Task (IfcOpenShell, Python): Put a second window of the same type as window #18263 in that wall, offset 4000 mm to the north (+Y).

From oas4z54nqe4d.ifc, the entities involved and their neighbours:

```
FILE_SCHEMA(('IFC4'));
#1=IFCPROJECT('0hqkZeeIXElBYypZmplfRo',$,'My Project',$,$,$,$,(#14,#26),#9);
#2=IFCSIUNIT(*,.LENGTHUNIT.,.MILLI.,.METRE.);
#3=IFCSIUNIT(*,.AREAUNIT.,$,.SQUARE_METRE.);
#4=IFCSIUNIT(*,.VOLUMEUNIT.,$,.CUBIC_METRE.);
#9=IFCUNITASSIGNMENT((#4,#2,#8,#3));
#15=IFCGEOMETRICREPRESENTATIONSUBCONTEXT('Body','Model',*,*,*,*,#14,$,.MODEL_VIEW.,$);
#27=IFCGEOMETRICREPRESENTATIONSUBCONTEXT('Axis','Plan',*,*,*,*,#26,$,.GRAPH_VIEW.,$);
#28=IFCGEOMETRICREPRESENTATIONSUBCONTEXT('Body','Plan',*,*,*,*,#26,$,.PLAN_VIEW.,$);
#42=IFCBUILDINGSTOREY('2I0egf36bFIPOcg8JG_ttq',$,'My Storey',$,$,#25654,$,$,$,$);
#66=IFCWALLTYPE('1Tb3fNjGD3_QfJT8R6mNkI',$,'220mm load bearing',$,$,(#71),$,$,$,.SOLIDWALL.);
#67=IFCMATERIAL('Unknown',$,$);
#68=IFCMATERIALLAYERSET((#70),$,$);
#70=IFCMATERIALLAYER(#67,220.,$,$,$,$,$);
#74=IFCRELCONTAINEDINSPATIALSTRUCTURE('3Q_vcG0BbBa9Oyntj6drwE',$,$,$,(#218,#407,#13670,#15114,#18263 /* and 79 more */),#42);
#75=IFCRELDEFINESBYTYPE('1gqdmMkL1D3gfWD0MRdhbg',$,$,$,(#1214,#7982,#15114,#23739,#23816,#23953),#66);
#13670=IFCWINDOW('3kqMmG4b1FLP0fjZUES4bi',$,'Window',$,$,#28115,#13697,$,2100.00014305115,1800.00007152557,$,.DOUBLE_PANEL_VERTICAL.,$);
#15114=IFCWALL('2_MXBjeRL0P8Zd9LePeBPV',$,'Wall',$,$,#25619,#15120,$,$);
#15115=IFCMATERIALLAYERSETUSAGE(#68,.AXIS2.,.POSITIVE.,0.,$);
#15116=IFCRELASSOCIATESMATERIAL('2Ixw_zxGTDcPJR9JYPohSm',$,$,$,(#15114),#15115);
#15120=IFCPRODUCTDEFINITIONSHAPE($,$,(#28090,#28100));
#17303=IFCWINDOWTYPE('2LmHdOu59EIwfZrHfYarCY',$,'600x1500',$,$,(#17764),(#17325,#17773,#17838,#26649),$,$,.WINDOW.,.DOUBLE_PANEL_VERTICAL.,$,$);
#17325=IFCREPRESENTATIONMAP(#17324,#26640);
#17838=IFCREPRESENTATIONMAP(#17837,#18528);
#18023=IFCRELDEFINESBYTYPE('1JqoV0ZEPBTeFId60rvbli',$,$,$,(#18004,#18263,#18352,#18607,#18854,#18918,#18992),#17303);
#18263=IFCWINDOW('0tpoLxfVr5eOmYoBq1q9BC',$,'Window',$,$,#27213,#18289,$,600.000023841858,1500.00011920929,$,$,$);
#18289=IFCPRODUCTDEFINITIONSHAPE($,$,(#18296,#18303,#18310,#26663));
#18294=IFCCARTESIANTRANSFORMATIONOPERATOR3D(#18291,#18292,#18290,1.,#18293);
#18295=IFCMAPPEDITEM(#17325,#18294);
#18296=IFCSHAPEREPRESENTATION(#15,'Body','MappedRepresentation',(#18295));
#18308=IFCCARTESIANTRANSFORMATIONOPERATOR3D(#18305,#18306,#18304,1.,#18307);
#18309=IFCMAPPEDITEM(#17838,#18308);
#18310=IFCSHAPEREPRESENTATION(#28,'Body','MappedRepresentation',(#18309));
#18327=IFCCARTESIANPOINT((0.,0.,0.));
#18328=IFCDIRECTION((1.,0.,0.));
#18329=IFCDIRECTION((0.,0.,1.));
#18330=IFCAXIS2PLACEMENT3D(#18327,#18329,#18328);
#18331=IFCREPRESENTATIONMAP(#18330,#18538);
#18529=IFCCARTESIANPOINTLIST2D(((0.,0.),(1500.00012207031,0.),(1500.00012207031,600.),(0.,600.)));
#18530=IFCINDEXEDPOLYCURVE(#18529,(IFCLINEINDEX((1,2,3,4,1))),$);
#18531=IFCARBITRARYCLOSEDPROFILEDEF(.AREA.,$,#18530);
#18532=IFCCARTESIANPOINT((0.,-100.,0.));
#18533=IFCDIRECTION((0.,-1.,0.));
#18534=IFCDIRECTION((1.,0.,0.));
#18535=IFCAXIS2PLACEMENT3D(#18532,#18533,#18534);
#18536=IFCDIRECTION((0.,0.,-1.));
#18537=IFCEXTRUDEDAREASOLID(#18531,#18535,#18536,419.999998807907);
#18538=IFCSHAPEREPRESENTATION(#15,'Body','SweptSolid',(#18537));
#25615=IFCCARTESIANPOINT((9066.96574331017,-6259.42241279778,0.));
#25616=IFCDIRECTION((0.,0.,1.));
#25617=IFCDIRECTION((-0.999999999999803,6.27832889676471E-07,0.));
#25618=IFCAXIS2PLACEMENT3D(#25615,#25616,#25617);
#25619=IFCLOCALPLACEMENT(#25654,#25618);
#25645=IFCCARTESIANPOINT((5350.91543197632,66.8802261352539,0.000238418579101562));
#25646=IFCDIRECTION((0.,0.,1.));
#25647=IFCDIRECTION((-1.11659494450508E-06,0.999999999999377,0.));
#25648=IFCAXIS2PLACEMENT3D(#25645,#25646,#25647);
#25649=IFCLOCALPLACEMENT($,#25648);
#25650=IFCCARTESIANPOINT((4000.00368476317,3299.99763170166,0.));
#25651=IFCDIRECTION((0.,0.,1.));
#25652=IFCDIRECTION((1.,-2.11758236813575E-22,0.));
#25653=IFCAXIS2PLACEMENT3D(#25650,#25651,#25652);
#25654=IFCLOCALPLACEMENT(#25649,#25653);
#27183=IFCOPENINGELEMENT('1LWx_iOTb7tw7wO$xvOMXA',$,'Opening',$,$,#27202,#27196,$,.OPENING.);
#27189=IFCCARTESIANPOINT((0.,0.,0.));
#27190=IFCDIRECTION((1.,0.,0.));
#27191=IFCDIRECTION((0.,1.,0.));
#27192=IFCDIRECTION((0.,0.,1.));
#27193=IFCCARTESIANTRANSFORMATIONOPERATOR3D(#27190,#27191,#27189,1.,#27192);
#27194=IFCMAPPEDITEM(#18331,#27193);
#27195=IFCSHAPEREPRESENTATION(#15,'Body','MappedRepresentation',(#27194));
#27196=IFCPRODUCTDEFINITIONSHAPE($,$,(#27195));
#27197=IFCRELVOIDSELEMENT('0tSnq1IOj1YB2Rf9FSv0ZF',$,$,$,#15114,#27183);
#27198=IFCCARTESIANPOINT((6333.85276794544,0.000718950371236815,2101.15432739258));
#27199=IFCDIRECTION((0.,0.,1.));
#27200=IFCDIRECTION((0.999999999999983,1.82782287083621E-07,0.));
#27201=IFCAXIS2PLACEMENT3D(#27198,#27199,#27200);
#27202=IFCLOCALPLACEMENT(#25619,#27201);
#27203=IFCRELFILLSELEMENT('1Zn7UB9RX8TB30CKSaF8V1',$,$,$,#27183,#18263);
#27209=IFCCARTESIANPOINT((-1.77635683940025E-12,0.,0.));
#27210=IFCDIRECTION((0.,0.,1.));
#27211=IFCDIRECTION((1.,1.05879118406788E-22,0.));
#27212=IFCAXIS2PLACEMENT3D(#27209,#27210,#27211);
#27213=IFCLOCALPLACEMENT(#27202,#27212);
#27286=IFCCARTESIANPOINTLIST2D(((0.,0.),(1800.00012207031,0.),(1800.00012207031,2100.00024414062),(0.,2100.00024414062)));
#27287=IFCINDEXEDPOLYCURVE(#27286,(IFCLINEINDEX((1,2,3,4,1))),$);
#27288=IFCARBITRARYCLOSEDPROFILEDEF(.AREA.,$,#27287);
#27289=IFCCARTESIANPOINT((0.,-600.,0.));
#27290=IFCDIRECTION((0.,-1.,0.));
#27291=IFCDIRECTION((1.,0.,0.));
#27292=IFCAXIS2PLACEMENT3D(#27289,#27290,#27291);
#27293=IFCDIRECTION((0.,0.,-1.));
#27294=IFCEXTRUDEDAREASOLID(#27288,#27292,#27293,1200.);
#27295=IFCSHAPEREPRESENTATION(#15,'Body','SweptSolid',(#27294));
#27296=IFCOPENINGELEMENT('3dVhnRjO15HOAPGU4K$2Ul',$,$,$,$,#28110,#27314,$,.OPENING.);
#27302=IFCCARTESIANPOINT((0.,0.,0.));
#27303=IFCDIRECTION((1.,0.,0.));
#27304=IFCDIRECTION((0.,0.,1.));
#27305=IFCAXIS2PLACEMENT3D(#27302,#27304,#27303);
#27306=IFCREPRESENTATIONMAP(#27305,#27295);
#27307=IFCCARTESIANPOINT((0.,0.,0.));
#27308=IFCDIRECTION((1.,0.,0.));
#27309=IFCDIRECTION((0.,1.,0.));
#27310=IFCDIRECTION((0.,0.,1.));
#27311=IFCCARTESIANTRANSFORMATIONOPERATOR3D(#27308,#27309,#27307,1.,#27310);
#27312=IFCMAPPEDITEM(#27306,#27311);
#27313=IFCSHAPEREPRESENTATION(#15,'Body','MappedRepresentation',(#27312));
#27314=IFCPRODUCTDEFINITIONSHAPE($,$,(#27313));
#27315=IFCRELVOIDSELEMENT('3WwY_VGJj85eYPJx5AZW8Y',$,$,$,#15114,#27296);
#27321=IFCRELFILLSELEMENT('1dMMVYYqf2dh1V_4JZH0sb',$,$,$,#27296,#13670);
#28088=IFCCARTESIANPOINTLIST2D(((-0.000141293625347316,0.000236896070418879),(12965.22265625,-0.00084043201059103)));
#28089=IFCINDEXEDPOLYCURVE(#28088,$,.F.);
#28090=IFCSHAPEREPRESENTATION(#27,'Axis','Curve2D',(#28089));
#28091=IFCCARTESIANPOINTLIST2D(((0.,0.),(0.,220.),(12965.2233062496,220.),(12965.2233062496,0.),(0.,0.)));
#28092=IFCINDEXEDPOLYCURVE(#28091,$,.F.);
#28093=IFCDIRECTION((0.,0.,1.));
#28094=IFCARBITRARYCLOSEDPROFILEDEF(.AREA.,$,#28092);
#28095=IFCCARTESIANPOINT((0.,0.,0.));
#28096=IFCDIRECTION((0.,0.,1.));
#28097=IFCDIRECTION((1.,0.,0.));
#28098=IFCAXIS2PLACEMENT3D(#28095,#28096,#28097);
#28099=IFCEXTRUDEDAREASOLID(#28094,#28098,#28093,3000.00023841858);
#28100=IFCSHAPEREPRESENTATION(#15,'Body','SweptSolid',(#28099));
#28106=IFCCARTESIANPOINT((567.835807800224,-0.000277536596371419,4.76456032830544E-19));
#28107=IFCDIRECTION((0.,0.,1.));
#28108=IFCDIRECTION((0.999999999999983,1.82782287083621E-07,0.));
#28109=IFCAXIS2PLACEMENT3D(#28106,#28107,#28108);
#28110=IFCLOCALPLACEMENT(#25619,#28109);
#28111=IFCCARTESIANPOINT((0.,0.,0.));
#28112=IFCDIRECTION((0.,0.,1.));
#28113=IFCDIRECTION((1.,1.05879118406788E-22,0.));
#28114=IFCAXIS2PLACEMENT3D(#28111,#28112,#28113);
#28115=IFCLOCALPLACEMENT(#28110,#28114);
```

```python
import ifcopenshell
import ifcopenshell.api.feature
import ifcopenshell.api.geometry
import ifcopenshell.api.root
import ifcopenshell.geom
import ifcopenshell.util.element
import ifcopenshell.util.placement
import ifcopenshell.util.shape
import ifcopenshell.util.unit

model = ifcopenshell.open("oas4z54nqe4d.ifc")
unit_scale = ifcopenshell.util.unit.calculate_unit_scale(model)
settings = ifcopenshell.geom.settings()


def volume(element):
    """Net volume in cubic metres, openings subtracted."""
    shape = ifcopenshell.geom.create_shape(settings, element)
    return ifcopenshell.util.shape.get_volume(shape.geometry)


window = model.by_guid("0tpoLxfVr5eOmYoBq1q9BC")
opening = window.FillsVoids[0].RelatingOpeningElement
wall = opening.VoidsElements[0].RelatingBuildingElement
before = volume(wall)
shift = ifcopenshell.util.placement.get_local_placement(wall.ObjectPlacement)[:3, 0] * -4 / unit_scale

# copy_class copies the void relationship, type, container and properties, but no geometry.
new_opening = ifcopenshell.api.root.copy_class(model, product=opening)
new_opening.Representation = ifcopenshell.util.element.copy_deep(
    model, opening.Representation, exclude=["IfcGeometricRepresentationContext", "IfcRepresentationMap"]
)
new_window = ifcopenshell.api.root.copy_class(model, product=window)
new_window.Representation = ifcopenshell.util.element.copy_deep(
    model, window.Representation, exclude=["IfcGeometricRepresentationContext", "IfcRepresentationMap"]
)
ifcopenshell.api.feature.add_filling(model, opening=new_opening, element=new_window)

for old, new in ((opening, new_opening), (window, new_window)):
    matrix = ifcopenshell.util.placement.get_local_placement(old.ObjectPlacement)
    matrix[:3, 3] += shift
    ifcopenshell.api.geometry.edit_object_placement(model, product=new, matrix=matrix, is_si=False)

after = volume(wall)

print(f"wall volume {before:.3f} -> {after:.3f} m3")

model.write("oas4z54nqe4d-out.ifc")
```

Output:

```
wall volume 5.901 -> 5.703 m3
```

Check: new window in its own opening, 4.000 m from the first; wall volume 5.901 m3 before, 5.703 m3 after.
